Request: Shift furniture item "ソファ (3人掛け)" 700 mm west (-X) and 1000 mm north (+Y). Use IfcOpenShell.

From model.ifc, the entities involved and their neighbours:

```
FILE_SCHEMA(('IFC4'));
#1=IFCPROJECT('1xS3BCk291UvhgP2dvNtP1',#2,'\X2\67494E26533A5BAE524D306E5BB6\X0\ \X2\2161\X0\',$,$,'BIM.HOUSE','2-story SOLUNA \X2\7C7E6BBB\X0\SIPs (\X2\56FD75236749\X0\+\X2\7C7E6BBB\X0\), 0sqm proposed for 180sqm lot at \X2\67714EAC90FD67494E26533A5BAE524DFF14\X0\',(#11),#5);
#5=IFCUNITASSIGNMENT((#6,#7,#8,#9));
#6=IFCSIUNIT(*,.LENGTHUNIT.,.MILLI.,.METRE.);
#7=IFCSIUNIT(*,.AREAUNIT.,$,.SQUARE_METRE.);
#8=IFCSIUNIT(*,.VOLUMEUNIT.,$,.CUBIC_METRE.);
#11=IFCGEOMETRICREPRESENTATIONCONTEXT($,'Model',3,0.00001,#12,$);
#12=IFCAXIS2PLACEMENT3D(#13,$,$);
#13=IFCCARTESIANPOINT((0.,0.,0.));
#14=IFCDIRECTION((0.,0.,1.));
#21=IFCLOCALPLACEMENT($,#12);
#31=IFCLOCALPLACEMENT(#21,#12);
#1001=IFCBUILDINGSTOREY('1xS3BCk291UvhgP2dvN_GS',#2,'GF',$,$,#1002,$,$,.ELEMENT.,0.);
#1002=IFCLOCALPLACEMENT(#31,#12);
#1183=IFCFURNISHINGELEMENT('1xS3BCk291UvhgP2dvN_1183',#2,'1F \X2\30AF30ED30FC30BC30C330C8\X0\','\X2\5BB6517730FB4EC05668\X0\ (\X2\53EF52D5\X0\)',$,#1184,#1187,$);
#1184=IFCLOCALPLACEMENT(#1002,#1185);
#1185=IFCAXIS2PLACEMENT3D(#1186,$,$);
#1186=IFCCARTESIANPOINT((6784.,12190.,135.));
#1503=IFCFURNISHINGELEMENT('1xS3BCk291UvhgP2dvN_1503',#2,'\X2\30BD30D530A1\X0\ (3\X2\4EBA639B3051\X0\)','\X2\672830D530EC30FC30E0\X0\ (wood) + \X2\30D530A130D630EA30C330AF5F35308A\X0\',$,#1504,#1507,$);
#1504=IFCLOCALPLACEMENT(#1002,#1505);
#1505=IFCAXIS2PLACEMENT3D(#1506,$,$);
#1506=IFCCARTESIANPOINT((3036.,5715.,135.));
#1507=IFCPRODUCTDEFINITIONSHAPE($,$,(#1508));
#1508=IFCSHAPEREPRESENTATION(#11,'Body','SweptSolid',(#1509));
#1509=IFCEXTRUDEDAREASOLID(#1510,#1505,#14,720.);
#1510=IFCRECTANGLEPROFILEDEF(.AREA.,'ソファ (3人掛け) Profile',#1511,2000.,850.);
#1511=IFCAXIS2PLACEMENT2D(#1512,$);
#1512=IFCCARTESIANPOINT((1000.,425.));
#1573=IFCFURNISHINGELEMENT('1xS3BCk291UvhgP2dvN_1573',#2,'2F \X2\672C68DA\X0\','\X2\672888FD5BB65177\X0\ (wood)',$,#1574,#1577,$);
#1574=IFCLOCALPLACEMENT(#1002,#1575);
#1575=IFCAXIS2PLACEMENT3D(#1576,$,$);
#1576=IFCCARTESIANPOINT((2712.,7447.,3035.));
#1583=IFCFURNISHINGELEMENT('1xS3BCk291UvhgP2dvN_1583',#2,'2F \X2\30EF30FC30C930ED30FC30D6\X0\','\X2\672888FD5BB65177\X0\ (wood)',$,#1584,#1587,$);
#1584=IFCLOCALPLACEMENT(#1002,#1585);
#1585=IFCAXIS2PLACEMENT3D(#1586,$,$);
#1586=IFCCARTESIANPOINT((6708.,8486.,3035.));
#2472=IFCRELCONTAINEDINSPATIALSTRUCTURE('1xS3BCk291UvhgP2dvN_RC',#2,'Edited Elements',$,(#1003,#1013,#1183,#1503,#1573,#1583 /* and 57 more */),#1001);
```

```python
import ifcopenshell
import ifcopenshell.api.geometry
import ifcopenshell.util.placement
import ifcopenshell.util.unit

model = ifcopenshell.open("model.ifc")
unit_scale = ifcopenshell.util.unit.calculate_unit_scale(model)

item = model.by_guid("1xS3BCk291UvhgP2dvN_1503")
matrix = ifcopenshell.util.placement.get_local_placement(item.ObjectPlacement)
matrix[0, 3] -= 0.7 / unit_scale
matrix[1, 3] += 1 / unit_scale
ifcopenshell.api.geometry.edit_object_placement(model, product=item, matrix=matrix, is_si=False)

print(ifcopenshell.util.placement.get_local_placement(item.ObjectPlacement).round(3) + 0.0)

model.write("model-out.ifc")
```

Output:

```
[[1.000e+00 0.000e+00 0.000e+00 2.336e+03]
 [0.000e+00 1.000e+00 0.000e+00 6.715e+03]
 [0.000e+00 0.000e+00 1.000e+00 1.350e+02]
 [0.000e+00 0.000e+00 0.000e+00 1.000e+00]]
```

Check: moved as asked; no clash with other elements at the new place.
